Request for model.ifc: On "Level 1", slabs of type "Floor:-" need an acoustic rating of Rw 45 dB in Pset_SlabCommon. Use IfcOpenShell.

First a look at what the model holds.

```python
import ifcopenshell
import ifcopenshell.util.element

model = ifcopenshell.open("model.ifc")
print(model.schema)
storey = next(s for s in model.by_type("IfcBuildingStorey") if s.Name == "Level 1")
slabs = [e for e in ifcopenshell.util.element.get_decomposition(storey) if e.is_a("IfcSlab")]
seen = {}
for e in slabs:
    element_type = ifcopenshell.util.element.get_type(e)
    key = (element_type.Name if element_type != e and element_type else None, ifcopenshell.util.element.get_pset(e, "Pset_SlabCommon", "AcousticRating"))
    seen[key] = seen.get(key, 0) + 1
for (name, value), count in sorted(seen.items(), key=str):
    print(count, "x", name, "|", value)
```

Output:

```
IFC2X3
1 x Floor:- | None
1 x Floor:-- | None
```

```python
import ifcopenshell
import ifcopenshell.api.pset
import ifcopenshell.util.element

model = ifcopenshell.open("model.ifc")

storey = next(s for s in model.by_type("IfcBuildingStorey") if s.Name == "Level 1")
slabs = [e for e in ifcopenshell.util.element.get_decomposition(storey) if e.is_a("IfcSlab")]

count = 0
for e in slabs:
    element_type = ifcopenshell.util.element.get_type(e)
    if element_type in (None, e) or element_type.Name != "Floor:-":
        continue
    # add_pset returns the element's existing set when there is one.
    pset = ifcopenshell.api.pset.add_pset(model, product=e, name="Pset_SlabCommon")
    ifcopenshell.api.pset.edit_pset(model, pset=pset, properties={"AcousticRating": "Rw 45 dB"})
    count += 1

print(count, "slabs updated")

model.write("model_edited.ifc")
```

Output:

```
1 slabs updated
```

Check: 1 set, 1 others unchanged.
